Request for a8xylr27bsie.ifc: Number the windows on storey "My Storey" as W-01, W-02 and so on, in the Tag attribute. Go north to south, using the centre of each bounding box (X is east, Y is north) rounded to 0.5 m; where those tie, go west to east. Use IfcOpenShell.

First a look at what the model holds.

```python
import ifcopenshell
import ifcopenshell.util.element
import ifcopenshell.util.placement

model = ifcopenshell.open("a8xylr27bsie.ifc")
print(model.schema)
storey = next(s for s in model.by_type("IfcBuildingStorey") if s.Name == "My Storey")
windows = [e for e in ifcopenshell.util.element.get_decomposition(storey) if e.is_a("IfcWindow")]
for e in sorted(windows, key=lambda e: e.id()):
    origin = ifcopenshell.util.placement.get_local_placement(e.ObjectPlacement)[:3, 3]
    print(e.id(), e.Tag, e.Name, origin.round(2) + 0.0, sep=" | ")
```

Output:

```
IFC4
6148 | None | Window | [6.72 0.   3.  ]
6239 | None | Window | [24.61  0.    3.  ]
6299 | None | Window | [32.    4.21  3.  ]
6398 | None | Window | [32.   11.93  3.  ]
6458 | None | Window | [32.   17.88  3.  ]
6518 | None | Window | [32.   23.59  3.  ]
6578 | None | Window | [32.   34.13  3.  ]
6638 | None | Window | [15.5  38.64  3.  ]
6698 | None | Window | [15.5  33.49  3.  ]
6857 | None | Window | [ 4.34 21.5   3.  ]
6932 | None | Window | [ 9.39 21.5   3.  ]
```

```python
import ifcopenshell
import ifcopenshell.geom
import ifcopenshell.util.element
import ifcopenshell.util.shape

model = ifcopenshell.open("a8xylr27bsie.ifc")
settings = ifcopenshell.geom.settings()
settings.set("use-world-coords", True)


def centre(element):
    shape = ifcopenshell.geom.create_shape(settings, element)
    return ifcopenshell.util.shape.get_bbox_centroid(shape.geometry)


storey = next(s for s in model.by_type("IfcBuildingStorey") if s.Name == "My Storey")
windows = [e for e in ifcopenshell.util.element.get_decomposition(storey) if e.is_a("IfcWindow")]

# Insertion points can sit at a corner or the storey origin, so sort by the geometry (in metres).
centres = {e: centre(e) for e in windows}
windows.sort(key=lambda e: (-round(centres[e][1] / 0.5), centres[e][0]))

for i, e in enumerate(windows, start=1):
    number = f"W-{i:02d}"
    e.Tag = number
    print(e.id(), number)

model.write("a8xylr27bsie_rev.ifc")
```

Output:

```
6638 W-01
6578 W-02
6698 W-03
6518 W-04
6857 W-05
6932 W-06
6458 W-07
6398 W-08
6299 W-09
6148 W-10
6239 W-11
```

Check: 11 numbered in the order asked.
